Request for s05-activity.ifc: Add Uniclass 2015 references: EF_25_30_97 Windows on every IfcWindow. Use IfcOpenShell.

First a look at what the model holds.

```python
import ifcopenshell

model = ifcopenshell.open("s05-activity.ifc")
print(model.schema)
print("classifications:", [c.Name for c in model.by_type("IfcClassification")])
for ifc_class in ("IfcDoor", "IfcRoof", "IfcStair", "IfcWall", "IfcWindow"):
    print(ifc_class, len(model.by_type(ifc_class)))
```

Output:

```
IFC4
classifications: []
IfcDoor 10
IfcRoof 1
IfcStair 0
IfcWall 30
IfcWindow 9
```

```python
import ifcopenshell
import ifcopenshell.api.classification

model = ifcopenshell.open("s05-activity.ifc")

system = ifcopenshell.api.classification.add_classification(model, classification="Uniclass 2015")

codes = {
    "IfcWindow": ("EF_25_30_97", "Windows"),
}
for ifc_class, (code, name) in codes.items():
    products = model.by_type(ifc_class)
    ifcopenshell.api.classification.add_reference(
        model, products=products, classification=system, identification=code, name=name
    )
    print(code, len(products))

model.write("s05-activity-out.ifc")
```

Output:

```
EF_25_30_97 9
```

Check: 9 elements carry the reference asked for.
